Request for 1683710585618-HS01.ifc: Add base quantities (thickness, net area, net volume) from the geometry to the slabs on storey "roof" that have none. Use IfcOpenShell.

First a look at what the model holds.

```python
import ifcopenshell
import ifcopenshell.util.element
import ifcopenshell.util.unit

model = ifcopenshell.open("1683710585618-HS01.ifc")
print(model.schema)
for unit_type in ("LENGTHUNIT", "AREAUNIT", "VOLUMEUNIT"):
    print(unit_type, ifcopenshell.util.unit.calculate_unit_scale(model, unit_type))
storey = next(s for s in model.by_type("IfcBuildingStorey") if s.Name == "roof")
slabs = [e for e in ifcopenshell.util.element.get_decomposition(storey) if e.is_a("IfcSlab")]
for e in sorted(slabs, key=lambda e: e.id()):
    print(e.id(), e.is_a(), e.Name, list(ifcopenshell.util.element.get_psets(e, qtos_only=True)), sep=" | ")
```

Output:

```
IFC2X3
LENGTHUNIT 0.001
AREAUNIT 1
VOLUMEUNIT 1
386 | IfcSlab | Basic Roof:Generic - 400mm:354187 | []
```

```python
import ifcopenshell
import ifcopenshell.api.pset
import ifcopenshell.geom
import ifcopenshell.util.element
import ifcopenshell.util.shape
import ifcopenshell.util.unit

model = ifcopenshell.open("1683710585618-HS01.ifc")
unit_scale = ifcopenshell.util.unit.calculate_unit_scale(model)
area_scale = ifcopenshell.util.unit.calculate_unit_scale(model, "AREAUNIT")
volume_scale = ifcopenshell.util.unit.calculate_unit_scale(model, "VOLUMEUNIT")
settings = ifcopenshell.geom.settings()

storey = next(s for s in model.by_type("IfcBuildingStorey") if s.Name == "roof")
slabs = [e for e in ifcopenshell.util.element.get_decomposition(storey) if e.is_a("IfcSlab")]

for e in sorted(slabs, key=lambda e: e.id()):
    if ifcopenshell.util.element.get_psets(e, qtos_only=True, should_inherit=False):
        continue
    # Geometry comes back in metres, in the element's own axes.
    shape = ifcopenshell.geom.create_shape(settings, e)
    values = {
        "Width": ifcopenshell.util.shape.get_z(shape.geometry) / unit_scale,
        "NetArea": ifcopenshell.util.shape.get_footprint_area(shape.geometry) / area_scale,
        "NetVolume": ifcopenshell.util.shape.get_volume(shape.geometry) / volume_scale,
    }
    qto = ifcopenshell.api.pset.add_qto(model, product=e, name="BaseQuantities")
    ifcopenshell.api.pset.edit_qto(model, qto=qto, properties=values)
    print(e.id(), {k: round(v, 3) for k, v in values.items()})

model.write("1683710585618-HS01_edited.ifc")
```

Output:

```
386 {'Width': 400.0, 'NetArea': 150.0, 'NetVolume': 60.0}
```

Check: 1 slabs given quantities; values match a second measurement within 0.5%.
